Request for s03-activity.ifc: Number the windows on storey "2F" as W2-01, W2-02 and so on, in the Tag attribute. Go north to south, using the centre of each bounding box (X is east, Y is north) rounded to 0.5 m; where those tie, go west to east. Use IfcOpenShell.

First a look at what the model holds.

```python
import ifcopenshell
import ifcopenshell.util.element
import ifcopenshell.util.placement

model = ifcopenshell.open("s03-activity.ifc")
print(model.schema)
storey = next(s for s in model.by_type("IfcBuildingStorey") if s.Name == "2F")
windows = [e for e in ifcopenshell.util.element.get_decomposition(storey) if e.is_a("IfcWindow")]
for e in sorted(windows, key=lambda e: e.id()):
    origin = ifcopenshell.util.placement.get_local_placement(e.ObjectPlacement)[:3, 3]
    print(e.id(), e.Tag, e.Name, origin.round(2) + 0.0, sep=" | ")
```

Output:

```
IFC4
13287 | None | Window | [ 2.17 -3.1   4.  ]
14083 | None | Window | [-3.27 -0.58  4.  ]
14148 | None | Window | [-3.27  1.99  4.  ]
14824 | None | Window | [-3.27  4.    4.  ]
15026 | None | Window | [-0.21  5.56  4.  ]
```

```python
import ifcopenshell
import ifcopenshell.geom
import ifcopenshell.util.element
import ifcopenshell.util.shape

model = ifcopenshell.open("s03-activity.ifc")
settings = ifcopenshell.geom.settings()
settings.set("use-world-coords", True)


def centre(element):
    shape = ifcopenshell.geom.create_shape(settings, element)
    return ifcopenshell.util.shape.get_bbox_centroid(shape.geometry)


storey = next(s for s in model.by_type("IfcBuildingStorey") if s.Name == "2F")
windows = [e for e in ifcopenshell.util.element.get_decomposition(storey) if e.is_a("IfcWindow")]

# Insertion points can sit at a corner or the storey origin, so sort by the geometry (in metres).
centres = {e: centre(e) for e in windows}
windows.sort(key=lambda e: (-round(centres[e][1] / 0.5), centres[e][0]))

for i, e in enumerate(windows, start=1):
    number = f"W2-{i:02d}"
    e.Tag = number
    print(e.id(), number)

model.write("s03-activity_updated.ifc")
```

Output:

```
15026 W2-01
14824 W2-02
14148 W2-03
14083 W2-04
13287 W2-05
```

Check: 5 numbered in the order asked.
